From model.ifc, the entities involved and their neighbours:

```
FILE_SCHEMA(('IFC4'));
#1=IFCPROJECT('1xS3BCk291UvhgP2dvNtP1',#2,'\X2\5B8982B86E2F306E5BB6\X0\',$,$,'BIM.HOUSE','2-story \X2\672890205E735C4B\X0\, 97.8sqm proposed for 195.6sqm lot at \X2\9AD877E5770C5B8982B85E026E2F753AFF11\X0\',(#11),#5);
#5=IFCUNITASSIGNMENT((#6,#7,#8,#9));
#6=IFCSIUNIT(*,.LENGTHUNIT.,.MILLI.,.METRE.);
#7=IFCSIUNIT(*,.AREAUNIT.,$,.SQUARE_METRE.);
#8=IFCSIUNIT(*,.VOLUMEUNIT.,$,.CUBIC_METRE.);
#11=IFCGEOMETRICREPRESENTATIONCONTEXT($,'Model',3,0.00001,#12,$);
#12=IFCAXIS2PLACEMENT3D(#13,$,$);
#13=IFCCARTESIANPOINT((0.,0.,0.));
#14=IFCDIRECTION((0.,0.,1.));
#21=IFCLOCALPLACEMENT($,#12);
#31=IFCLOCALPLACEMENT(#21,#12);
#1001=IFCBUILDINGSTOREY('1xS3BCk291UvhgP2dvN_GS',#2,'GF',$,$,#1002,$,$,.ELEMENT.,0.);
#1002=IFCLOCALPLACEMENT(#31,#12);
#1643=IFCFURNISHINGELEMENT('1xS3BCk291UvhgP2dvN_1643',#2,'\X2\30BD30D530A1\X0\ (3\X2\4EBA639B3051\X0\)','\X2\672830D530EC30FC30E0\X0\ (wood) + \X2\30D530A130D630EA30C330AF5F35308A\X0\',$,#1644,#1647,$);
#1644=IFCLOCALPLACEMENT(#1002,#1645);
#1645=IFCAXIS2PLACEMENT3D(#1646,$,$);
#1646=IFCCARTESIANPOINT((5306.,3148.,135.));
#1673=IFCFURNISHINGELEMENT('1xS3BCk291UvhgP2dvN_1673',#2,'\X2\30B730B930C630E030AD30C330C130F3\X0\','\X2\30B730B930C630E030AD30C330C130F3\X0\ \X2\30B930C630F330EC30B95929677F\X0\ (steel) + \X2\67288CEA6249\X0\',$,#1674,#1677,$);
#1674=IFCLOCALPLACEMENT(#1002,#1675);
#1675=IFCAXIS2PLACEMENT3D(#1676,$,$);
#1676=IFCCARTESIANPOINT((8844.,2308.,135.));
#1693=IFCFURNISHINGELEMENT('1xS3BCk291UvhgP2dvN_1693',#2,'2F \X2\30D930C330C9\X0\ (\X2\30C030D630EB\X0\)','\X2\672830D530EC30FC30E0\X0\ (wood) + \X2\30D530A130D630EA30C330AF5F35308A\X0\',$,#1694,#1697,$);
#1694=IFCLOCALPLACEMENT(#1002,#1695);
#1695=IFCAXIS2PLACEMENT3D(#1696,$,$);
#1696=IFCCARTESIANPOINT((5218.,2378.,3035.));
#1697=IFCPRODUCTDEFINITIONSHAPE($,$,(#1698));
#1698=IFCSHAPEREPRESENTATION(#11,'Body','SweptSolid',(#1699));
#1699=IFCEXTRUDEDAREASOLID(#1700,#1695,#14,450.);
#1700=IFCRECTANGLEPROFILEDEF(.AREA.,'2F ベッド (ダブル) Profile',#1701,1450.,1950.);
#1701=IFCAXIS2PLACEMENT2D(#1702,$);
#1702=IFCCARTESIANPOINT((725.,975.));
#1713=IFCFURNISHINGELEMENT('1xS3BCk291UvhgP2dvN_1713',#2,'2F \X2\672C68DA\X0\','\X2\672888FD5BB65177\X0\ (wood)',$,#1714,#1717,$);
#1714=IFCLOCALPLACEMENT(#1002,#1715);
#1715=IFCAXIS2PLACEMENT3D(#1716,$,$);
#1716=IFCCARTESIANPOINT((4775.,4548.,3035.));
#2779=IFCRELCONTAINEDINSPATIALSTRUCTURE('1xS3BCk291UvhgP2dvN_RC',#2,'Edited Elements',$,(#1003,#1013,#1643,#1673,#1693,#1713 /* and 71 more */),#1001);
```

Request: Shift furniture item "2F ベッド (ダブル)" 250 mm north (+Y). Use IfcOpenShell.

```python
import ifcopenshell
import ifcopenshell.api.geometry
import ifcopenshell.util.placement
import ifcopenshell.util.unit

model = ifcopenshell.open("model.ifc")
unit_scale = ifcopenshell.util.unit.calculate_unit_scale(model)

item = model.by_guid("1xS3BCk291UvhgP2dvN_1693")
matrix = ifcopenshell.util.placement.get_local_placement(item.ObjectPlacement)
matrix[1, 3] += 0.25 / unit_scale
ifcopenshell.api.geometry.edit_object_placement(model, product=item, matrix=matrix, is_si=False)

print(ifcopenshell.util.placement.get_local_placement(item.ObjectPlacement).round(3) + 0.0)

model.write("model_updated.ifc")
```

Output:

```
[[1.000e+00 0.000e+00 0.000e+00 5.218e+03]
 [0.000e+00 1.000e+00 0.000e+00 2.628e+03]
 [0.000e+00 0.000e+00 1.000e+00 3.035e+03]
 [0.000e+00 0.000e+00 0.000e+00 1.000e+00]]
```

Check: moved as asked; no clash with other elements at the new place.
